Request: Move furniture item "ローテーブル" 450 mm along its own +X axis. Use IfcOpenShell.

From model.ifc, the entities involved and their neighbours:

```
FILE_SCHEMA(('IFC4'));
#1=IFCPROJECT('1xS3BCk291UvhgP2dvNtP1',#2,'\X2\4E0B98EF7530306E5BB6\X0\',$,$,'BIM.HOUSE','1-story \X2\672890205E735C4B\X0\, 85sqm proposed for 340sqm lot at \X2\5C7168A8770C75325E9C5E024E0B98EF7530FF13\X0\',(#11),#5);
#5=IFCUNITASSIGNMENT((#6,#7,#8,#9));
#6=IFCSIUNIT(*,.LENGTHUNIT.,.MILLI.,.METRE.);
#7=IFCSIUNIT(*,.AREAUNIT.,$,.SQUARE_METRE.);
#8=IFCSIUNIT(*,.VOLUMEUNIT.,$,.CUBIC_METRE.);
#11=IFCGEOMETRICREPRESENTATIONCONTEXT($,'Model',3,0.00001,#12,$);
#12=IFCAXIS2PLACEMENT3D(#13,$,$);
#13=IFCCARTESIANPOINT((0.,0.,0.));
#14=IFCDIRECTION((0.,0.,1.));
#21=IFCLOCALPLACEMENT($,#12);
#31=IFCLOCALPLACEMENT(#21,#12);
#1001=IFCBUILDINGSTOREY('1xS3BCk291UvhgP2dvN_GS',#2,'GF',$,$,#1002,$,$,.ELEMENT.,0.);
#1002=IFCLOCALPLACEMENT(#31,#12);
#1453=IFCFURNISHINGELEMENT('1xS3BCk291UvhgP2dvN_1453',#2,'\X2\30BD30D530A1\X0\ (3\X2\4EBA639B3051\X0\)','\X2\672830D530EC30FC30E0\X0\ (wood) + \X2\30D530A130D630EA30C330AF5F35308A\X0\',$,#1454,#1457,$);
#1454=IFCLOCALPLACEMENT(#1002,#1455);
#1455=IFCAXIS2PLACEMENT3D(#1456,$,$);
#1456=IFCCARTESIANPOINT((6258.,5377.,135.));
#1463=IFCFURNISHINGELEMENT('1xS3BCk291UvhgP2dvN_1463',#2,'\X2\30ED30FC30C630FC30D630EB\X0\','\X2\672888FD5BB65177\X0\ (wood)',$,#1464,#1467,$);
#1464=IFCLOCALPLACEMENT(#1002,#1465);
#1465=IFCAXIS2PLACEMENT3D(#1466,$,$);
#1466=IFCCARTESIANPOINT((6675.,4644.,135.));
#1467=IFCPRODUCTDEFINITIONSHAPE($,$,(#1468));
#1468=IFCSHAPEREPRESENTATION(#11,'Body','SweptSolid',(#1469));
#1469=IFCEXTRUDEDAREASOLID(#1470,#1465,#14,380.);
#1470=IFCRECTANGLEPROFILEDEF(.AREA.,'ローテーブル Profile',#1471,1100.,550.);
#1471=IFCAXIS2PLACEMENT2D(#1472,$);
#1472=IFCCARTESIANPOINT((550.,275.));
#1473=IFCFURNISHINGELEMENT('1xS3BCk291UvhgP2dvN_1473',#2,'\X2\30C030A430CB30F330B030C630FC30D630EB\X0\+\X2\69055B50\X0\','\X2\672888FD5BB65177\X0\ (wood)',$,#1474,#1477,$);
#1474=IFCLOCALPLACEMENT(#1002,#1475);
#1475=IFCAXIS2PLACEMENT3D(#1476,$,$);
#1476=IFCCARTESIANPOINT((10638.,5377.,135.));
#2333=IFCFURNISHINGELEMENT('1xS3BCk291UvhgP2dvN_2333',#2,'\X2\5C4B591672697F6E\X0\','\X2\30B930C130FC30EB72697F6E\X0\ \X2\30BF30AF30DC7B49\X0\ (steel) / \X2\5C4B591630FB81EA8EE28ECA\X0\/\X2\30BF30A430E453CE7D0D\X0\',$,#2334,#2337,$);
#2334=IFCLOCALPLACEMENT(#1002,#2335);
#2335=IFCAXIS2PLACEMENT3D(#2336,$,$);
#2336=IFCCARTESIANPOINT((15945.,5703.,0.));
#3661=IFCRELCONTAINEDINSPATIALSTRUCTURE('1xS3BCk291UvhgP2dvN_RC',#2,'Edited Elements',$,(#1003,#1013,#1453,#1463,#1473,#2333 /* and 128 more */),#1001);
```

```python
import ifcopenshell
import ifcopenshell.api.geometry
import ifcopenshell.util.placement
import ifcopenshell.util.unit

model = ifcopenshell.open("model.ifc")
unit_scale = ifcopenshell.util.unit.calculate_unit_scale(model)

item = model.by_guid("1xS3BCk291UvhgP2dvN_1463")
matrix = ifcopenshell.util.placement.get_local_placement(item.ObjectPlacement)
matrix[:3, 3] += matrix[:3, 0] * 0.45 / unit_scale
ifcopenshell.api.geometry.edit_object_placement(model, product=item, matrix=matrix, is_si=False)

print(ifcopenshell.util.placement.get_local_placement(item.ObjectPlacement).round(3) + 0.0)

model.write("model_v2.ifc")
```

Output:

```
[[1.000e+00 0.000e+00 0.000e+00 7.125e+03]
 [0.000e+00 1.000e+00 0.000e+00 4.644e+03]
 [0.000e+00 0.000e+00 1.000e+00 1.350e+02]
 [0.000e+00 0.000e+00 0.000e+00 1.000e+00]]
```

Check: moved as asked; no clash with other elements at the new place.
